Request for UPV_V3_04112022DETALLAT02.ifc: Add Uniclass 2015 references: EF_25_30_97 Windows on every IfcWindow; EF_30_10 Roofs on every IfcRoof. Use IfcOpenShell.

First a look at what the model holds.

```python
import ifcopenshell

model = ifcopenshell.open("UPV_V3_04112022DETALLAT02.ifc")
print(model.schema)
print("classifications:", [c.Name for c in model.by_type("IfcClassification")])
for ifc_class in ("IfcDoor", "IfcRoof", "IfcStair", "IfcWall", "IfcWindow"):
    print(ifc_class, len(model.by_type(ifc_class)))
```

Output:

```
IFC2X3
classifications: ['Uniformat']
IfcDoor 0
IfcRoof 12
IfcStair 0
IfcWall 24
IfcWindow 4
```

```python
import ifcopenshell
import ifcopenshell.api.classification

model = ifcopenshell.open("UPV_V3_04112022DETALLAT02.ifc")

# IFC2X3 requires Source and Edition and has no link from the project to the system.
system = model.create_entity("IfcClassification", Source="NBS", Edition="2015", Name="Uniclass 2015")

codes = {
    "IfcWindow": ("EF_25_30_97", "Windows"),
    "IfcRoof": ("EF_30_10", "Roofs"),
}
for ifc_class, (code, name) in codes.items():
    products = model.by_type(ifc_class)
    ifcopenshell.api.classification.add_reference(
        model, products=products, classification=system, identification=code, name=name
    )
    print(code, len(products))

model.write("UPV_V3_04112022DETALLAT02_updated.ifc")
```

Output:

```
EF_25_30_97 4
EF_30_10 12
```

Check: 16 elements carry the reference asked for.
